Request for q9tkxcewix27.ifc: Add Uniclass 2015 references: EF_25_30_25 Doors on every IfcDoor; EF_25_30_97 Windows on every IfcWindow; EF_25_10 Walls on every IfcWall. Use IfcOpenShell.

First a look at what the model holds.

```python
import ifcopenshell

model = ifcopenshell.open("q9tkxcewix27.ifc")
print(model.schema)
print("classifications:", [c.Name for c in model.by_type("IfcClassification")])
for ifc_class in ("IfcDoor", "IfcRoof", "IfcStair", "IfcWall", "IfcWindow"):
    print(ifc_class, len(model.by_type(ifc_class)))
```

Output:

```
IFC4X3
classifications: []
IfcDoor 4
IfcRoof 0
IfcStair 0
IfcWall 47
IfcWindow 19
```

```python
import ifcopenshell
import ifcopenshell.api.classification

model = ifcopenshell.open("q9tkxcewix27.ifc")

system = ifcopenshell.api.classification.add_classification(model, classification="Uniclass 2015")

codes = {
    "IfcDoor": ("EF_25_30_25", "Doors"),
    "IfcWindow": ("EF_25_30_97", "Windows"),
    "IfcWall": ("EF_25_10", "Walls"),
}
for ifc_class, (code, name) in codes.items():
    products = model.by_type(ifc_class)
    ifcopenshell.api.classification.add_reference(
        model, products=products, classification=system, identification=code, name=name
    )
    print(code, len(products))

model.write("q9tkxcewix27_edited.ifc")
```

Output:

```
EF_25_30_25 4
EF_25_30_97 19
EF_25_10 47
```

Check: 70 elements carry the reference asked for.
